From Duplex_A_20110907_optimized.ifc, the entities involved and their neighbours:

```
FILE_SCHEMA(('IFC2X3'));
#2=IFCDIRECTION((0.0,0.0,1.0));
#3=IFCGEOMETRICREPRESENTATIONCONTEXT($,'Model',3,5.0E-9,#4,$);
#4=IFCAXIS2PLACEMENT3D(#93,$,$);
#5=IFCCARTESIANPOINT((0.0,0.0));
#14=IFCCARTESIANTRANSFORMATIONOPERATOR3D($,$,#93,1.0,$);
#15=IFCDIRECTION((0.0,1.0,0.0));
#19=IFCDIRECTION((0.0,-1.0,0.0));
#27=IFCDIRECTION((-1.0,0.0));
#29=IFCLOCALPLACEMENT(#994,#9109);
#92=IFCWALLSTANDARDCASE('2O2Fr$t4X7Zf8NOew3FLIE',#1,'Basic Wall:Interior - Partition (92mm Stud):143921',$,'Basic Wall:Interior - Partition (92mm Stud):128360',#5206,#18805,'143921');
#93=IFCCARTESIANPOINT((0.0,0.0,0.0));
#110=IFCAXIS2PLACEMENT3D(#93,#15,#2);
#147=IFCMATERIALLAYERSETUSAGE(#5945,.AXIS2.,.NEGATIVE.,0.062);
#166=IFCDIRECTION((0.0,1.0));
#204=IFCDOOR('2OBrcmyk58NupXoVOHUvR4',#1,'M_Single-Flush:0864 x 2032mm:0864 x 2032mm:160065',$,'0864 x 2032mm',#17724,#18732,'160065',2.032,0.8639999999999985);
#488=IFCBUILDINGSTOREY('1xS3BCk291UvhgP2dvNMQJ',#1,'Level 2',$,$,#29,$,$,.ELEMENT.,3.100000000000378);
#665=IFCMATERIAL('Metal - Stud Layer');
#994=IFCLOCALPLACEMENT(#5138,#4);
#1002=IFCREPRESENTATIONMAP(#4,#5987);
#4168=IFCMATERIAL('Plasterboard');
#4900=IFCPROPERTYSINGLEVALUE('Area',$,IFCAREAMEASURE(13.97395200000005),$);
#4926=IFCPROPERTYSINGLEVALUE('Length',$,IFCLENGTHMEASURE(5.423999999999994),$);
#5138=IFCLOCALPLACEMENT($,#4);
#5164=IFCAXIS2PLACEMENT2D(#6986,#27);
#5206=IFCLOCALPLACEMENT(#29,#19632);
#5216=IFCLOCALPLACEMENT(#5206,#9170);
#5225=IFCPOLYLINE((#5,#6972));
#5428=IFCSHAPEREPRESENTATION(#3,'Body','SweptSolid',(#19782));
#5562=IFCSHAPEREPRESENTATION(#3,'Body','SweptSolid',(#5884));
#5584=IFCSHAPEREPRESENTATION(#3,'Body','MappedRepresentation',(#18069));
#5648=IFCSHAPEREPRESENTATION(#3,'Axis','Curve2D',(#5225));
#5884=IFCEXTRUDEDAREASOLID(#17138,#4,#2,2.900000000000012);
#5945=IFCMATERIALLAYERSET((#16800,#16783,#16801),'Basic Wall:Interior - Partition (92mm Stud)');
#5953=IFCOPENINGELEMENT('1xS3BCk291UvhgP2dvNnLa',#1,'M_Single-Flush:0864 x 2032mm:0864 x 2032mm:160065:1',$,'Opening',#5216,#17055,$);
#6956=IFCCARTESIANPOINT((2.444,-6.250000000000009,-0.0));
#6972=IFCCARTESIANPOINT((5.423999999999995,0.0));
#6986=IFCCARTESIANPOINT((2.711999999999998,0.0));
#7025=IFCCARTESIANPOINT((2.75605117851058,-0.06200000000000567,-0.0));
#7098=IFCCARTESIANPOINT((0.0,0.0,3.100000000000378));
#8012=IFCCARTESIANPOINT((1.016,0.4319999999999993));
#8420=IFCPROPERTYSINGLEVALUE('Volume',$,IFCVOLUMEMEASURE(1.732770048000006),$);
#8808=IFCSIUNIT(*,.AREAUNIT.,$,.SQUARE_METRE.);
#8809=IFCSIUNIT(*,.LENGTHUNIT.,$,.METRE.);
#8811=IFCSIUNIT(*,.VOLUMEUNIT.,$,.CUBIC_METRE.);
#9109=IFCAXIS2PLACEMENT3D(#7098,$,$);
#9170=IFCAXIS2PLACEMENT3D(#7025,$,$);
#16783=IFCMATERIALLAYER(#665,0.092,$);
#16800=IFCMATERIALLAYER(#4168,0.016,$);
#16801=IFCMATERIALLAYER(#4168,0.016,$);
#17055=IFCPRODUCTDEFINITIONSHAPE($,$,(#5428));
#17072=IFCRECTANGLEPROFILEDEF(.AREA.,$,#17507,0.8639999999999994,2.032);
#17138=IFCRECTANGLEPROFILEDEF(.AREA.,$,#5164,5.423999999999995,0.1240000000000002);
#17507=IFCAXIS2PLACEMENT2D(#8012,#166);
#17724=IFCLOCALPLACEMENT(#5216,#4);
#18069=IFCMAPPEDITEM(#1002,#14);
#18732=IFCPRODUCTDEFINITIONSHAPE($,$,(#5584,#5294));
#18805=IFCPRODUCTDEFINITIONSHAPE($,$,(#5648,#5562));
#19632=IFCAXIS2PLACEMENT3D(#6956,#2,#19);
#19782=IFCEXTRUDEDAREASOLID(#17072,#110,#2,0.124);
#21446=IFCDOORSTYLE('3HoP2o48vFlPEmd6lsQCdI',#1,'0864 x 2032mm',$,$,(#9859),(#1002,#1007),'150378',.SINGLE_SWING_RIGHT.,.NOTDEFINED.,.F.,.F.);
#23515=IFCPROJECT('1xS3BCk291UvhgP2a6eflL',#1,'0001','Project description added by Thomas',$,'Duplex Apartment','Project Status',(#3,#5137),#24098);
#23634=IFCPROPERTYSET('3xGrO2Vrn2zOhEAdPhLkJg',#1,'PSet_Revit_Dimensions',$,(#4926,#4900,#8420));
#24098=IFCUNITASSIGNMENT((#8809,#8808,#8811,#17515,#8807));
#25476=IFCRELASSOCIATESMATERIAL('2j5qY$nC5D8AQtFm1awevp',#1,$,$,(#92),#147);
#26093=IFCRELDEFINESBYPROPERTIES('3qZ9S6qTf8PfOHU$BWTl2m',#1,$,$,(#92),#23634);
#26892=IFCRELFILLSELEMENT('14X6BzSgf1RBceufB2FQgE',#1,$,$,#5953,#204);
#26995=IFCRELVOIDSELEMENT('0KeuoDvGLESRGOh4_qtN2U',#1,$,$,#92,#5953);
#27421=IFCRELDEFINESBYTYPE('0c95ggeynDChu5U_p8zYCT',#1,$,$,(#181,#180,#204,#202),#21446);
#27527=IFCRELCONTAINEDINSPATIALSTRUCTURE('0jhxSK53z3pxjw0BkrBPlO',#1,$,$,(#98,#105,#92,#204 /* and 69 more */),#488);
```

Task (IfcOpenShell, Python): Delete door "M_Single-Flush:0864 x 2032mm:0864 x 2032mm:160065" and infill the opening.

```python
import ifcopenshell
import ifcopenshell.api.feature
import ifcopenshell.api.pset
import ifcopenshell.api.root
import ifcopenshell.geom
import ifcopenshell.util.element
import ifcopenshell.util.shape
import ifcopenshell.util.unit

model = ifcopenshell.open("Duplex_A_20110907_optimized.ifc")
area_scale = ifcopenshell.util.unit.calculate_unit_scale(model, "AREAUNIT")
volume_scale = ifcopenshell.util.unit.calculate_unit_scale(model, "VOLUMEUNIT")
settings = ifcopenshell.geom.settings()


def volume(element):
    """Net volume in cubic metres, openings subtracted."""
    shape = ifcopenshell.geom.create_shape(settings, element)
    return ifcopenshell.util.shape.get_volume(shape.geometry)


door = model.by_id(204)
opening = door.FillsVoids[0].RelatingOpeningElement
wall = opening.VoidsElements[0].RelatingBuildingElement
before = volume(wall)

ifcopenshell.api.root.remove_product(model, product=door)
ifcopenshell.api.feature.remove_feature(model, feature=opening)

after = volume(wall)
thickness = 0.124  # wall thickness in metres

# Update the wall's stored quantities.
pset = model.by_id(ifcopenshell.util.element.get_pset(wall, "PSet_Revit_Dimensions", should_inherit=False)["id"])
ifcopenshell.api.pset.edit_pset(model, pset=pset, properties={
    "Area": model.create_entity("IfcAreaMeasure", after / thickness / area_scale),
    "Volume": model.create_entity("IfcVolumeMeasure", after / volume_scale),
})

print(f"wall volume {before:.3f} -> {after:.3f} m3")

model.write("Duplex_A_20110907_optimized_edited.ifc")
```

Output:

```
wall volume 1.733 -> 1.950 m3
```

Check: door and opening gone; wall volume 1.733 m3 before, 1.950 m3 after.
